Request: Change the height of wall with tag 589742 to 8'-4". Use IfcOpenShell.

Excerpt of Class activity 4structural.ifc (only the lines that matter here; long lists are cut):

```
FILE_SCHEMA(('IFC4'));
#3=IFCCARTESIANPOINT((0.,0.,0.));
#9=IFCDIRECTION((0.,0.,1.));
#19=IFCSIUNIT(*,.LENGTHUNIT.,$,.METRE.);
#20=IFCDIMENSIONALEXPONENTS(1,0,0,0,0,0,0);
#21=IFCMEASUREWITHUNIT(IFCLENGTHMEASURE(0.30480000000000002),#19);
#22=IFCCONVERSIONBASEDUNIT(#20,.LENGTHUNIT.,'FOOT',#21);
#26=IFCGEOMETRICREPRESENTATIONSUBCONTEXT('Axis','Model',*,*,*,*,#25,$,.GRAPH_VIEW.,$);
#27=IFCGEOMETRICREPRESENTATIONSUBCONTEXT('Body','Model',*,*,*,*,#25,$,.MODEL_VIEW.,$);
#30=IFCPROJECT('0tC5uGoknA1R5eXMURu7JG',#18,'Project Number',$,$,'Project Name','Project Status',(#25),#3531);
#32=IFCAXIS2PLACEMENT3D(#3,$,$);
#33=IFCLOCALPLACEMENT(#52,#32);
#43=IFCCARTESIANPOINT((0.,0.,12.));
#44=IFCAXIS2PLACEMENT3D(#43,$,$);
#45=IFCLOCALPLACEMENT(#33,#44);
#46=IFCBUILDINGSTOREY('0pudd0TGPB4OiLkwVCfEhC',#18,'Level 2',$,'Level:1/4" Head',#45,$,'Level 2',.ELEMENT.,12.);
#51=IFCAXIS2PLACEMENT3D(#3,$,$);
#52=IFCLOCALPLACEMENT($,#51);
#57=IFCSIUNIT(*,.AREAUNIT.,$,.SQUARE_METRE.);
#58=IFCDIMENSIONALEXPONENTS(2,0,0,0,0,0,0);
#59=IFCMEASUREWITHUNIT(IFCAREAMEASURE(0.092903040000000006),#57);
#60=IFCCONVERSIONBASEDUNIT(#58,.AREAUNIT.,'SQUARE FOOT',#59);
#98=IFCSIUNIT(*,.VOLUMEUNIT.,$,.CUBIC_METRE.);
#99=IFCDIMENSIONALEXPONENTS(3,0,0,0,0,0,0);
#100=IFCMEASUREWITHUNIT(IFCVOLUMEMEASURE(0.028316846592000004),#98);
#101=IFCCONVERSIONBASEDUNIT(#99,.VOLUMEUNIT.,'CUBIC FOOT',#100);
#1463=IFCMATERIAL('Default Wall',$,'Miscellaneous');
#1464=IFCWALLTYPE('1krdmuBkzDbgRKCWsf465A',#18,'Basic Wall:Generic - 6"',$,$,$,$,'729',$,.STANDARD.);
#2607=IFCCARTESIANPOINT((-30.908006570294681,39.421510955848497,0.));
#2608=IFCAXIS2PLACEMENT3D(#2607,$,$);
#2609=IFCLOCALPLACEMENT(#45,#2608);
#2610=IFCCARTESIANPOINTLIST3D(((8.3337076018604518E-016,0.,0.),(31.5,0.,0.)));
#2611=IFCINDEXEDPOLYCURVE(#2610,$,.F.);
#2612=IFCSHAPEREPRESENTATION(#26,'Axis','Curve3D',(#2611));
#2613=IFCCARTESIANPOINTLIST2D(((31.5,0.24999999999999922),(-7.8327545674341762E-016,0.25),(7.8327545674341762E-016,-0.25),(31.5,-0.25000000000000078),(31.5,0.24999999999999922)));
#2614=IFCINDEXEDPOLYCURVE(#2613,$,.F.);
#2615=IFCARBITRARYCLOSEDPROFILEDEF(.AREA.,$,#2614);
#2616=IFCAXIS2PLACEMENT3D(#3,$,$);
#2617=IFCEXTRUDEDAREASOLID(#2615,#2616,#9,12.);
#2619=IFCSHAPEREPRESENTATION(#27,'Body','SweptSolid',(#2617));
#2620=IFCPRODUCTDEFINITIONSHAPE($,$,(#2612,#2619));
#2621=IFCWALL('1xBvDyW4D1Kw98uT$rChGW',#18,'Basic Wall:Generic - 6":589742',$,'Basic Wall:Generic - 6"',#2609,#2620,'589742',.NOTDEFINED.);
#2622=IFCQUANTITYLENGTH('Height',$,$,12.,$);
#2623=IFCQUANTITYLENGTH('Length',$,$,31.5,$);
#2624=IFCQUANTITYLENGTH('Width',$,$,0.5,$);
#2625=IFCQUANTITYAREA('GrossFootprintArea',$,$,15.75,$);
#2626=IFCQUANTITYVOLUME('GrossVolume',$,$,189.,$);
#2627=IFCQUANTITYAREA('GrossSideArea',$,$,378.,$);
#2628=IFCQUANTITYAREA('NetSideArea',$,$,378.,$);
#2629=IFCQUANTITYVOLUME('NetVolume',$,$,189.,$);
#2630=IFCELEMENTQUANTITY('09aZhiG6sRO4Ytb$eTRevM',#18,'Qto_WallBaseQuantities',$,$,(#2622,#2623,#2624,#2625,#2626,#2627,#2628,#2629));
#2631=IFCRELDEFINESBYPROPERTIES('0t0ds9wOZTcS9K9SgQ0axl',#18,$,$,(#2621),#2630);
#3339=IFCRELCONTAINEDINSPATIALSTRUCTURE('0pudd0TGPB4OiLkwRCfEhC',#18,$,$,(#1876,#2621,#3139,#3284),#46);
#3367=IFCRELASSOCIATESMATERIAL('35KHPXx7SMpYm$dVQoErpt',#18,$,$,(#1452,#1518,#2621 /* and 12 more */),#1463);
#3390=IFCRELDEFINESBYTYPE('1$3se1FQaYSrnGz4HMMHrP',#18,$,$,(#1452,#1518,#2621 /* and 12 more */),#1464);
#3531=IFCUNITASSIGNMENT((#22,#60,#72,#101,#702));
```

```python
import ifcopenshell
import ifcopenshell.api.pset
import ifcopenshell.geom
import ifcopenshell.util.element
import ifcopenshell.util.representation
import ifcopenshell.util.shape
import ifcopenshell.util.unit

model = ifcopenshell.open("Class activity 4structural.ifc")
unit_scale = ifcopenshell.util.unit.calculate_unit_scale(model)
area_scale = ifcopenshell.util.unit.calculate_unit_scale(model, "AREAUNIT")
volume_scale = ifcopenshell.util.unit.calculate_unit_scale(model, "VOLUMEUNIT")
settings = ifcopenshell.geom.settings()


def volume(element):
    """Net volume in cubic metres, openings subtracted."""
    shape = ifcopenshell.geom.create_shape(settings, element)
    return ifcopenshell.util.shape.get_volume(shape.geometry)


wall = model.by_id(2621)
before = volume(wall)

body = ifcopenshell.util.representation.get_representation(wall, "Model", "Body")
solid = body.Items[0]
old_height = solid.Depth
solid.Depth = 100 * 0.0254 / unit_scale
after = volume(wall)
thickness = 0.1524  # wall thickness in metres

# Update the stored height, areas and volumes.
qto = model.by_id(ifcopenshell.util.element.get_pset(wall, "Qto_WallBaseQuantities", should_inherit=False)["id"])
ifcopenshell.api.pset.edit_qto(model, qto=qto, properties={
    "Height": solid.Depth,
    "GrossVolume": ifcopenshell.util.element.get_pset(wall, "Qto_WallBaseQuantities", "GrossVolume") * solid.Depth / old_height,
    "GrossSideArea": ifcopenshell.util.element.get_pset(wall, "Qto_WallBaseQuantities", "GrossSideArea") * solid.Depth / old_height,
    "NetSideArea": after / thickness / area_scale,
    "NetVolume": after / volume_scale,
})

print(f"height {old_height:g} -> {solid.Depth:g}, volume {before:.3f} -> {after:.3f} m3")

model.write("Class activity 4structural_v2.ifc")
```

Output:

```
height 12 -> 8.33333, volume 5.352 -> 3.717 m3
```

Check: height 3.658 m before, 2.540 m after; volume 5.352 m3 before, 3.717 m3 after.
